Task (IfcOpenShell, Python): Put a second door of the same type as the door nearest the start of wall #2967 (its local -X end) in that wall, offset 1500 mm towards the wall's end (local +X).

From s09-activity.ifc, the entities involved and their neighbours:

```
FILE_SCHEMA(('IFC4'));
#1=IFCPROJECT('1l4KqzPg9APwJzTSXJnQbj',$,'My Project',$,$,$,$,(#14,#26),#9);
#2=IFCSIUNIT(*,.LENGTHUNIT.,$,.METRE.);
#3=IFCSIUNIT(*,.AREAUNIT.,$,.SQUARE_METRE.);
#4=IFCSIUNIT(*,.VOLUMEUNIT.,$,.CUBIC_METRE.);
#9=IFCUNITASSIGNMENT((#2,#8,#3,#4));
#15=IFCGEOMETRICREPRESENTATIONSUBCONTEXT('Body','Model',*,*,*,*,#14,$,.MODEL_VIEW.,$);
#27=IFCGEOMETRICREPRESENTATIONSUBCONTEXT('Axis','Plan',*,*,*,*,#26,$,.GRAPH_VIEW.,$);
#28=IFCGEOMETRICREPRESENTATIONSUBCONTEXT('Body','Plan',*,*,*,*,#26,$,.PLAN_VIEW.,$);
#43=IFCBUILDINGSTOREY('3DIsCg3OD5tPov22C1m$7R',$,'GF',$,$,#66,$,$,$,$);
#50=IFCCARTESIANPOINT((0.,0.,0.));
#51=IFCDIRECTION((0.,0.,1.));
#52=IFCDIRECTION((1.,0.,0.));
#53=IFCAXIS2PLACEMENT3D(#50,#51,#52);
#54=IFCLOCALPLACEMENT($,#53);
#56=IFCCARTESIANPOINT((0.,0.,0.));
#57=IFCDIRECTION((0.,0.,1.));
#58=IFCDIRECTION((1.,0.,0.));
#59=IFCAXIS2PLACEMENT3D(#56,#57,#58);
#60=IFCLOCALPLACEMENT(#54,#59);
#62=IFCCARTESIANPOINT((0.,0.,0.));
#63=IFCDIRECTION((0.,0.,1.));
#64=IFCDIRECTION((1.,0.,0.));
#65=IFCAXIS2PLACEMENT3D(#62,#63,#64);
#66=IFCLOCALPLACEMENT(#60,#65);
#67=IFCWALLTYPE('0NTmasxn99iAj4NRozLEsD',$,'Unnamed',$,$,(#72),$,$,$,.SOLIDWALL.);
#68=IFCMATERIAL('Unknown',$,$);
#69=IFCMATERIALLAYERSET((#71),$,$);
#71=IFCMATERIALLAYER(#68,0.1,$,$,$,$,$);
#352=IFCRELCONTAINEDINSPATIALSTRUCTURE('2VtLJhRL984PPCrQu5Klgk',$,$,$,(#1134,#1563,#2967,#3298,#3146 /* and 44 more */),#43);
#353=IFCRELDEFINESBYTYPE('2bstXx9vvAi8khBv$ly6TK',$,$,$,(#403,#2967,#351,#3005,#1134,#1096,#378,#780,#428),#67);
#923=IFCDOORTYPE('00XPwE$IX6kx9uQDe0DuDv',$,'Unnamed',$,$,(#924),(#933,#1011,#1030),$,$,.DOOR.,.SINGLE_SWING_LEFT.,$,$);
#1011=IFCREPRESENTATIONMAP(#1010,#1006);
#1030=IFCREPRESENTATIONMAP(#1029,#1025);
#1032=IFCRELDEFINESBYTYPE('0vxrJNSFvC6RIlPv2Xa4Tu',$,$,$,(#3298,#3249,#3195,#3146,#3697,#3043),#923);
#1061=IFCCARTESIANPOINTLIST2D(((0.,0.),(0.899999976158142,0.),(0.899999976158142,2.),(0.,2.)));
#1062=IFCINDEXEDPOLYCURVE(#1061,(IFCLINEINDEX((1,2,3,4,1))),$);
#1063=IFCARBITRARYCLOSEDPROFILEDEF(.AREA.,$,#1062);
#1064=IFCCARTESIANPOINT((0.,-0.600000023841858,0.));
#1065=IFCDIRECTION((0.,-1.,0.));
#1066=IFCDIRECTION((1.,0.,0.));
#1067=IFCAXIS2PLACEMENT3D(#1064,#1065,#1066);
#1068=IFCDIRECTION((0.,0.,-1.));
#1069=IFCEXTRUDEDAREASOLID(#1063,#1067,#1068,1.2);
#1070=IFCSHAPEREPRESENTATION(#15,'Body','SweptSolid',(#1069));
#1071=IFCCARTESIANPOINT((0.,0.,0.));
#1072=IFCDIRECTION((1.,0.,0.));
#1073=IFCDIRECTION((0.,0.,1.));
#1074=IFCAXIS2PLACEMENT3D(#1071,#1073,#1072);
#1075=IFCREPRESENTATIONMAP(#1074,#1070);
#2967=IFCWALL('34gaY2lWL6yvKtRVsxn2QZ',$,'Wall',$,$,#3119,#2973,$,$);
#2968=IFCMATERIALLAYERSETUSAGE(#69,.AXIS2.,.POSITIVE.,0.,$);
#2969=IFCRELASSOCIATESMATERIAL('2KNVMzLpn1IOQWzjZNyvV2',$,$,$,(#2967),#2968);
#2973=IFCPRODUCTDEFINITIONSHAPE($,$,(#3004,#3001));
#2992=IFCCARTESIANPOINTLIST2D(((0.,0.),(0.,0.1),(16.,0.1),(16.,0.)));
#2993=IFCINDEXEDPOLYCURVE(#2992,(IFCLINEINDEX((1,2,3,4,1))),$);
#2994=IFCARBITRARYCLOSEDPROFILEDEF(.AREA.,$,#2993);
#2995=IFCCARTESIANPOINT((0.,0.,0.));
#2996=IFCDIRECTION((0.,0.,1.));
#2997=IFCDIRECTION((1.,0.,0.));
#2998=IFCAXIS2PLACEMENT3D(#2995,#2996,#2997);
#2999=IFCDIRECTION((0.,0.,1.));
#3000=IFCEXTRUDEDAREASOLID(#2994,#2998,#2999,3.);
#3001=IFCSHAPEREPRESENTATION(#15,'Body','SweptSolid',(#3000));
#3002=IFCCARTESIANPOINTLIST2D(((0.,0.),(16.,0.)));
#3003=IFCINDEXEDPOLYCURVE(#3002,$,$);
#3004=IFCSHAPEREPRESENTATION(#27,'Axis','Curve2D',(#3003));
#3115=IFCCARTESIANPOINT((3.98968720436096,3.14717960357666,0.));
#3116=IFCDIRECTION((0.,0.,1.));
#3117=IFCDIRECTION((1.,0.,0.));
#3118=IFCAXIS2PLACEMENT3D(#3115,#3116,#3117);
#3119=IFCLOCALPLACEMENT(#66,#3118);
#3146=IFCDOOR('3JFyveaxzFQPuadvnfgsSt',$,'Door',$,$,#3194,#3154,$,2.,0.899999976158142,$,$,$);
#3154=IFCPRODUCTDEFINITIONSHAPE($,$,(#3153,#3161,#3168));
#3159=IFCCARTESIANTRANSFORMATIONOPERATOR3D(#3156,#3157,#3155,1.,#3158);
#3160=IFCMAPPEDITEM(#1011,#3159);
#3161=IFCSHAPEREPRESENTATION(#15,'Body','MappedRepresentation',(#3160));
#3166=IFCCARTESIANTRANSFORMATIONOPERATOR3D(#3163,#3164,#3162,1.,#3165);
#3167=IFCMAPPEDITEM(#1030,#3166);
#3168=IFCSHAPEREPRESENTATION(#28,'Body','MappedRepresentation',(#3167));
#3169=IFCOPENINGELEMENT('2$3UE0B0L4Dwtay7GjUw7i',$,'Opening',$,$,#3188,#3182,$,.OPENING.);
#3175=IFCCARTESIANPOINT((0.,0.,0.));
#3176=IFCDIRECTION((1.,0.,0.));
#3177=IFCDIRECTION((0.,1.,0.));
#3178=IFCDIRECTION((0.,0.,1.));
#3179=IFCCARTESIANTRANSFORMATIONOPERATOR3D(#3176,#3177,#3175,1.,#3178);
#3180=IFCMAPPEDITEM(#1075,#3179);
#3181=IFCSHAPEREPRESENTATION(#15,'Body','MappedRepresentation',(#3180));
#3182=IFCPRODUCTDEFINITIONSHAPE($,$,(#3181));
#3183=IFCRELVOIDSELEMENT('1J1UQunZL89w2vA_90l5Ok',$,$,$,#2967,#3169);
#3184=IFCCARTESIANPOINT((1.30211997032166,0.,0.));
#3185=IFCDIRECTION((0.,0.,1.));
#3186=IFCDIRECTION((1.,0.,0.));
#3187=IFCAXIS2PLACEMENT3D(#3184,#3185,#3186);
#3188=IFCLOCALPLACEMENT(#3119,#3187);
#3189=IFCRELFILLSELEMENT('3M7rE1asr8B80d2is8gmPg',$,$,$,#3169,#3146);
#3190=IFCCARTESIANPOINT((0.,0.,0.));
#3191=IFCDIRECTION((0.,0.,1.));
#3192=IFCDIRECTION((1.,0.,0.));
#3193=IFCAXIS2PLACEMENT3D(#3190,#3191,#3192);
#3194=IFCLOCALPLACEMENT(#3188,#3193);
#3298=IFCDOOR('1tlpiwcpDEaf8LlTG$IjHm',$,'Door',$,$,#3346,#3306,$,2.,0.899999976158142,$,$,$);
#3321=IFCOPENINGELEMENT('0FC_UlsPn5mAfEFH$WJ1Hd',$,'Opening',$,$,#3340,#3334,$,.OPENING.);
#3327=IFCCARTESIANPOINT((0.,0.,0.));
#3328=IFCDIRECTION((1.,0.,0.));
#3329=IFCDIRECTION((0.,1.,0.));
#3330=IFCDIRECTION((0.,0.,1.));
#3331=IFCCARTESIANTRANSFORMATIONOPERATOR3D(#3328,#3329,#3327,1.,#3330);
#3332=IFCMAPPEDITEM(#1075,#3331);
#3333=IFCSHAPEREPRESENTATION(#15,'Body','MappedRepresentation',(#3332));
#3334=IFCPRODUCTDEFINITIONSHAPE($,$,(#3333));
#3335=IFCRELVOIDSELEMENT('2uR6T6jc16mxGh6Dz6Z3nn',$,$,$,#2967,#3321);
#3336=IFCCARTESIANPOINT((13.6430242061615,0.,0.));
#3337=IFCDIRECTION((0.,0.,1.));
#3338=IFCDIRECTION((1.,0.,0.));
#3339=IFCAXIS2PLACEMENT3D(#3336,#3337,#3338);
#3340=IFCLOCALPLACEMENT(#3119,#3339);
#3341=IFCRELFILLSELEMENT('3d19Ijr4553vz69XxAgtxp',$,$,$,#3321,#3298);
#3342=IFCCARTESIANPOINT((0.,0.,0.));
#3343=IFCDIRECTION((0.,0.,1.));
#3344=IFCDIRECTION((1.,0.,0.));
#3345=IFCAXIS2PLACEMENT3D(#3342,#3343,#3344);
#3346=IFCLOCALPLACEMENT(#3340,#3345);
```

```python
import ifcopenshell
import ifcopenshell.api.feature
import ifcopenshell.api.geometry
import ifcopenshell.api.root
import ifcopenshell.geom
import ifcopenshell.util.element
import ifcopenshell.util.placement
import ifcopenshell.util.shape
import ifcopenshell.util.unit

model = ifcopenshell.open("s09-activity.ifc")
unit_scale = ifcopenshell.util.unit.calculate_unit_scale(model)
settings = ifcopenshell.geom.settings()


def volume(element):
    """Net volume in cubic metres, openings subtracted."""
    shape = ifcopenshell.geom.create_shape(settings, element)
    return ifcopenshell.util.shape.get_volume(shape.geometry)


door = model.by_guid("3JFyveaxzFQPuadvnfgsSt")
opening = door.FillsVoids[0].RelatingOpeningElement
wall = opening.VoidsElements[0].RelatingBuildingElement
before = volume(wall)
shift = ifcopenshell.util.placement.get_local_placement(wall.ObjectPlacement)[:3, 0] * 1.5 / unit_scale

# copy_class copies the void relationship, type, container and properties, but no geometry.
new_opening = ifcopenshell.api.root.copy_class(model, product=opening)
new_opening.Representation = ifcopenshell.util.element.copy_deep(
    model, opening.Representation, exclude=["IfcGeometricRepresentationContext", "IfcRepresentationMap"]
)
new_door = ifcopenshell.api.root.copy_class(model, product=door)
new_door.Representation = ifcopenshell.util.element.copy_deep(
    model, door.Representation, exclude=["IfcGeometricRepresentationContext", "IfcRepresentationMap"]
)
ifcopenshell.api.feature.add_filling(model, opening=new_opening, element=new_door)

for old, new in ((opening, new_opening), (door, new_door)):
    matrix = ifcopenshell.util.placement.get_local_placement(old.ObjectPlacement)
    matrix[:3, 3] += shift
    ifcopenshell.api.geometry.edit_object_placement(model, product=new, matrix=matrix, is_si=False)

after = volume(wall)

print(f"wall volume {before:.3f} -> {after:.3f} m3")

model.write("s09-activity_v2.ifc")
```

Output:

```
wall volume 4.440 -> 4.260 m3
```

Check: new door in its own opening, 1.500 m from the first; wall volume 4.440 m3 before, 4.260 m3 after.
